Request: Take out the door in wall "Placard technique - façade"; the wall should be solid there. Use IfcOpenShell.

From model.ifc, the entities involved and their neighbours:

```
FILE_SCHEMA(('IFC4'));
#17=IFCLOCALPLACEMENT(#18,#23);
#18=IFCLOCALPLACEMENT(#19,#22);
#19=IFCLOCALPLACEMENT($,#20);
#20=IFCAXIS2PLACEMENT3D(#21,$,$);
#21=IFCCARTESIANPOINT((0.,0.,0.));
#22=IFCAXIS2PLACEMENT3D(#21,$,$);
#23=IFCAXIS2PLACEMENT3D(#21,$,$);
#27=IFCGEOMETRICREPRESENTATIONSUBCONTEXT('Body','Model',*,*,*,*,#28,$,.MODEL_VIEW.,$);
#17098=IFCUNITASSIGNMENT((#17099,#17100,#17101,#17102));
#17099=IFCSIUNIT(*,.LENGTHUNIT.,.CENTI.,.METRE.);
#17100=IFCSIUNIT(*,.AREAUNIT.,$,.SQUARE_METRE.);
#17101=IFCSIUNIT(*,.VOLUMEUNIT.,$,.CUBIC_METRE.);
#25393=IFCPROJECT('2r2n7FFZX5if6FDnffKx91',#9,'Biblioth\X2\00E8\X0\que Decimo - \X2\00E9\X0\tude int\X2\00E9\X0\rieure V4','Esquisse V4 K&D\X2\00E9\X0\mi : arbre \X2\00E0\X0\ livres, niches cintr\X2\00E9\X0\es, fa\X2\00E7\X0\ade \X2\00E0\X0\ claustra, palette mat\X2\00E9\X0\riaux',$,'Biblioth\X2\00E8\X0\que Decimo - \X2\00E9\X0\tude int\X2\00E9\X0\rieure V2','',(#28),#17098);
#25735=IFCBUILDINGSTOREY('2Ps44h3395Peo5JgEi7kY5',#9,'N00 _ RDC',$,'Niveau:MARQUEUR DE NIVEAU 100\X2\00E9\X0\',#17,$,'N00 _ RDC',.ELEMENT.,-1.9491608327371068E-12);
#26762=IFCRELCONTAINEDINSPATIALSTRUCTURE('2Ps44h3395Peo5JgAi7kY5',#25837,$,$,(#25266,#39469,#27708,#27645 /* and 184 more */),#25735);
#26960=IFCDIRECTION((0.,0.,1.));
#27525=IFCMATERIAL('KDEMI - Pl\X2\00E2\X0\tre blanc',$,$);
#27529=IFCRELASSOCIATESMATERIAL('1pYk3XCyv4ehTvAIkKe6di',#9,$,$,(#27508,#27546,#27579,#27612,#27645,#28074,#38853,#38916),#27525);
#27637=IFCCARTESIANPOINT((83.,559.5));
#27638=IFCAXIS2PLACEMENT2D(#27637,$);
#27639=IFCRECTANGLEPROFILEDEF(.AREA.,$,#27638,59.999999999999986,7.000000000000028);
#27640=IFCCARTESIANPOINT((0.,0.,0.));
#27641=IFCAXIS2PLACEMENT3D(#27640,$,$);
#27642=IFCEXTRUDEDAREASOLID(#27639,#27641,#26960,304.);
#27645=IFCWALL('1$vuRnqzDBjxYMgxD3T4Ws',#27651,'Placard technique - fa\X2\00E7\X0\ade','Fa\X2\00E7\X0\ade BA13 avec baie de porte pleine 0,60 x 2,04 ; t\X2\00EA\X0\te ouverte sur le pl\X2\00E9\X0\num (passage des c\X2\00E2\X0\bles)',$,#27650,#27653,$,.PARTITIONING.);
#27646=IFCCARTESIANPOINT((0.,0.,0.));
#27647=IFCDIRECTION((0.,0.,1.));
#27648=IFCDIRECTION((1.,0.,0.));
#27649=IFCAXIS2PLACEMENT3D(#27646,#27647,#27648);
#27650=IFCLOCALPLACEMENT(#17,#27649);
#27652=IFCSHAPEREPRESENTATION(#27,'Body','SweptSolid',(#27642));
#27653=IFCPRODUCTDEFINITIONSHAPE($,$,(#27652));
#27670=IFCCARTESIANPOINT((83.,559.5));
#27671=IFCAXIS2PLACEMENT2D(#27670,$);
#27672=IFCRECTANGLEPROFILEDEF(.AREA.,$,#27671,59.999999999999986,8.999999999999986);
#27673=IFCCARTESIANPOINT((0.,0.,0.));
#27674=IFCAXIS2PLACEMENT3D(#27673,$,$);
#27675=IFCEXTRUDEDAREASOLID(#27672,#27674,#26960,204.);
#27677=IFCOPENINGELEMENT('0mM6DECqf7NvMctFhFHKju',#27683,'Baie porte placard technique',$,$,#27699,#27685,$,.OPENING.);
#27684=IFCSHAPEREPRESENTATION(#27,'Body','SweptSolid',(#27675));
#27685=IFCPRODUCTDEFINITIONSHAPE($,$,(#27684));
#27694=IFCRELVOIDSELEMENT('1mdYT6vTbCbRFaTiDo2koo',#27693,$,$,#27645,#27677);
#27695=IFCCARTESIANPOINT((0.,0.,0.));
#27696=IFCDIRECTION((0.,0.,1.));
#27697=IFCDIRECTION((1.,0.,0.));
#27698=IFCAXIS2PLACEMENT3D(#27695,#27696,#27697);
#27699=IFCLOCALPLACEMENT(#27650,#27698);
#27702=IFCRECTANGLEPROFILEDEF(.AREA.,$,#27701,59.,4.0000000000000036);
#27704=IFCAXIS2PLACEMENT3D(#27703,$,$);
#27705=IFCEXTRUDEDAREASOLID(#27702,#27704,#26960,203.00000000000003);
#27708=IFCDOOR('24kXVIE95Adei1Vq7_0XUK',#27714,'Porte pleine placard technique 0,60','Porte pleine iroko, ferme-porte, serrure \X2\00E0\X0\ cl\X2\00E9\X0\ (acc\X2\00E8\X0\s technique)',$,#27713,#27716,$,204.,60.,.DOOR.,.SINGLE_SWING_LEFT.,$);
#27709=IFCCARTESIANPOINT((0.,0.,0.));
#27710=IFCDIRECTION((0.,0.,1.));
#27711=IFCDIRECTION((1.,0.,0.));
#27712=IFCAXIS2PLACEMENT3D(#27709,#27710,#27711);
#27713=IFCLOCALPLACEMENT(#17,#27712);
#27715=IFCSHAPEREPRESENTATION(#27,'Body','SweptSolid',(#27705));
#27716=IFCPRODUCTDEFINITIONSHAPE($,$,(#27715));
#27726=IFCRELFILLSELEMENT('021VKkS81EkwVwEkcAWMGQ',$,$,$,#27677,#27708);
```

```python
import ifcopenshell
import ifcopenshell.api.feature
import ifcopenshell.api.root
import ifcopenshell.geom
import ifcopenshell.util.shape

model = ifcopenshell.open("model.ifc")
settings = ifcopenshell.geom.settings()


def volume(element):
    """Net volume in cubic metres, openings subtracted."""
    shape = ifcopenshell.geom.create_shape(settings, element)
    return ifcopenshell.util.shape.get_volume(shape.geometry)


door = model.by_guid("24kXVIE95Adei1Vq7_0XUK")
opening = door.FillsVoids[0].RelatingOpeningElement
wall = opening.VoidsElements[0].RelatingBuildingElement
before = volume(wall)

ifcopenshell.api.root.remove_product(model, product=door)
ifcopenshell.api.feature.remove_feature(model, feature=opening)

after = volume(wall)

print(f"wall volume {before:.3f} -> {after:.3f} m3")

model.write("model_edited.ifc")
```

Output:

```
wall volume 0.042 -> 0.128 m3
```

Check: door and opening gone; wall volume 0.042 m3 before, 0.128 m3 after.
